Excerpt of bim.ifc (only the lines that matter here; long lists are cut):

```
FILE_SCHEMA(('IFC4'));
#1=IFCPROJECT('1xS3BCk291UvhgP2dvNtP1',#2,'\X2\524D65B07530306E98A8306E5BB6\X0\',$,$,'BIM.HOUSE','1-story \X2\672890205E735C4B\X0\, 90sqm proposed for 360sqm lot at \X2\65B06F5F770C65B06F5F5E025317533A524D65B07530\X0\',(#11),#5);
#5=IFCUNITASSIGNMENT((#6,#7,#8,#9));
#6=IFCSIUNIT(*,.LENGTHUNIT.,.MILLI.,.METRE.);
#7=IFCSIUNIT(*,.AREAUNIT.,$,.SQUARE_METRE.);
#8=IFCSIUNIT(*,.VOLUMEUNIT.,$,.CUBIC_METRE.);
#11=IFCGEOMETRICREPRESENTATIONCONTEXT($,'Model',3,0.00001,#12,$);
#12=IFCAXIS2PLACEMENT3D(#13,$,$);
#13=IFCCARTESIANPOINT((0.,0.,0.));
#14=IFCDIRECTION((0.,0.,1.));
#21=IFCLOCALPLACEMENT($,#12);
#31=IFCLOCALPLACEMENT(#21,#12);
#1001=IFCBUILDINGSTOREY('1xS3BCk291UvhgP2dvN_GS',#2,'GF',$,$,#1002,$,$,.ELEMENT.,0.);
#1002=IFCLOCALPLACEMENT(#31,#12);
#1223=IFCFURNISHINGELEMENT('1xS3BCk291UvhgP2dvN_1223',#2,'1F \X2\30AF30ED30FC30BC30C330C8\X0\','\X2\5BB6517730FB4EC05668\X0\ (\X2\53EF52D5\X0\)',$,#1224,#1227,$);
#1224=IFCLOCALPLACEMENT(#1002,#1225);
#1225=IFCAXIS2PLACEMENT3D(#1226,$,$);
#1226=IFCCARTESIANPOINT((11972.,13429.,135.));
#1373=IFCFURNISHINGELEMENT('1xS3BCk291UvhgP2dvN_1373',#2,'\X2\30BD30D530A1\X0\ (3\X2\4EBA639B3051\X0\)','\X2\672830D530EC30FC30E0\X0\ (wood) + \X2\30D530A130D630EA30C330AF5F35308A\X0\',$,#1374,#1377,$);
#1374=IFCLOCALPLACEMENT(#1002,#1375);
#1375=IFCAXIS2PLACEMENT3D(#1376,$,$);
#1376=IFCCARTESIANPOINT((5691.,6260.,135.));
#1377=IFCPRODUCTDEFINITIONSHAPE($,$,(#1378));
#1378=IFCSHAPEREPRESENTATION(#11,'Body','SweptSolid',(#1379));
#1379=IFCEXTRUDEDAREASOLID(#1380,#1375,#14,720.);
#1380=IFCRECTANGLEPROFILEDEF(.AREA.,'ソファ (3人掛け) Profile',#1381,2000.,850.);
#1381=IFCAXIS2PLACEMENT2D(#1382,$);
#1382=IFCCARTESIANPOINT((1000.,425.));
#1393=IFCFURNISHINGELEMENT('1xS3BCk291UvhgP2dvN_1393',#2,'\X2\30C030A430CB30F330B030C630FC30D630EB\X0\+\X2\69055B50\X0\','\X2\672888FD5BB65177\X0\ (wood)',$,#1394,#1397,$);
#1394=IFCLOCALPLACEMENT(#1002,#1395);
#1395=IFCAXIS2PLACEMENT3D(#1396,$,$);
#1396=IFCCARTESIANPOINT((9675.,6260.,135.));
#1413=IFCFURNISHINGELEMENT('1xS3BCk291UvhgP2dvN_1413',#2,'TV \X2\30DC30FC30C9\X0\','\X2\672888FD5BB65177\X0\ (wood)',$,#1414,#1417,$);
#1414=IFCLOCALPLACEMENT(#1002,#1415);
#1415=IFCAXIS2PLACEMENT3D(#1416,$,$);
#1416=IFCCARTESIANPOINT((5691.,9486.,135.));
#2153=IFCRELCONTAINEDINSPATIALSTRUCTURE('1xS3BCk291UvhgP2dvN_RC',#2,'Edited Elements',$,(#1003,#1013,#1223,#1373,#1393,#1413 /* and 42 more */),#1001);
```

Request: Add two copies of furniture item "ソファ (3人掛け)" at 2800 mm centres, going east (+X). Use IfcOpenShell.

```python
import numpy as np
import ifcopenshell
import ifcopenshell.api.geometry
import ifcopenshell.api.root
import ifcopenshell.util.element
import ifcopenshell.util.placement
import ifcopenshell.util.unit

model = ifcopenshell.open("bim.ifc")
unit_scale = ifcopenshell.util.unit.calculate_unit_scale(model)


def reuse_history(source, copy):
    """copy_class also copies each property set's owner history, people and application; keep the originals."""
    for rel in copy.IsDefinedBy:
        if rel.is_a("IfcRelDefinesByProperties") and (history := rel.RelatingPropertyDefinition.OwnerHistory):
            rel.RelatingPropertyDefinition.OwnerHistory = source.OwnerHistory
            ifcopenshell.util.element.remove_deep2(model, history)


source = model.by_guid("1xS3BCk291UvhgP2dvN_1373")
base = ifcopenshell.util.placement.get_local_placement(source.ObjectPlacement)
step = np.array([1.0, 0.0, 0.0]) * 2.8 / unit_scale

for i in range(1, 3):
    copy = ifcopenshell.api.root.copy_class(model, product=source)
    copy.Representation = ifcopenshell.util.element.copy_deep(
        model, source.Representation, exclude=["IfcGeometricRepresentationContext", "IfcRepresentationMap"]
    )
    reuse_history(source, copy)
    matrix = base.copy()
    matrix[:3, 3] += i * step
    print("added at", matrix[:3, 3].round(3) + 0.0)
    ifcopenshell.api.geometry.edit_object_placement(model, product=copy, matrix=matrix, is_si=False)

model.write("bim_updated.ifc")
```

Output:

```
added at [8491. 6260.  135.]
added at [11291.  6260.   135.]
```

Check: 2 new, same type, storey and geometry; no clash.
